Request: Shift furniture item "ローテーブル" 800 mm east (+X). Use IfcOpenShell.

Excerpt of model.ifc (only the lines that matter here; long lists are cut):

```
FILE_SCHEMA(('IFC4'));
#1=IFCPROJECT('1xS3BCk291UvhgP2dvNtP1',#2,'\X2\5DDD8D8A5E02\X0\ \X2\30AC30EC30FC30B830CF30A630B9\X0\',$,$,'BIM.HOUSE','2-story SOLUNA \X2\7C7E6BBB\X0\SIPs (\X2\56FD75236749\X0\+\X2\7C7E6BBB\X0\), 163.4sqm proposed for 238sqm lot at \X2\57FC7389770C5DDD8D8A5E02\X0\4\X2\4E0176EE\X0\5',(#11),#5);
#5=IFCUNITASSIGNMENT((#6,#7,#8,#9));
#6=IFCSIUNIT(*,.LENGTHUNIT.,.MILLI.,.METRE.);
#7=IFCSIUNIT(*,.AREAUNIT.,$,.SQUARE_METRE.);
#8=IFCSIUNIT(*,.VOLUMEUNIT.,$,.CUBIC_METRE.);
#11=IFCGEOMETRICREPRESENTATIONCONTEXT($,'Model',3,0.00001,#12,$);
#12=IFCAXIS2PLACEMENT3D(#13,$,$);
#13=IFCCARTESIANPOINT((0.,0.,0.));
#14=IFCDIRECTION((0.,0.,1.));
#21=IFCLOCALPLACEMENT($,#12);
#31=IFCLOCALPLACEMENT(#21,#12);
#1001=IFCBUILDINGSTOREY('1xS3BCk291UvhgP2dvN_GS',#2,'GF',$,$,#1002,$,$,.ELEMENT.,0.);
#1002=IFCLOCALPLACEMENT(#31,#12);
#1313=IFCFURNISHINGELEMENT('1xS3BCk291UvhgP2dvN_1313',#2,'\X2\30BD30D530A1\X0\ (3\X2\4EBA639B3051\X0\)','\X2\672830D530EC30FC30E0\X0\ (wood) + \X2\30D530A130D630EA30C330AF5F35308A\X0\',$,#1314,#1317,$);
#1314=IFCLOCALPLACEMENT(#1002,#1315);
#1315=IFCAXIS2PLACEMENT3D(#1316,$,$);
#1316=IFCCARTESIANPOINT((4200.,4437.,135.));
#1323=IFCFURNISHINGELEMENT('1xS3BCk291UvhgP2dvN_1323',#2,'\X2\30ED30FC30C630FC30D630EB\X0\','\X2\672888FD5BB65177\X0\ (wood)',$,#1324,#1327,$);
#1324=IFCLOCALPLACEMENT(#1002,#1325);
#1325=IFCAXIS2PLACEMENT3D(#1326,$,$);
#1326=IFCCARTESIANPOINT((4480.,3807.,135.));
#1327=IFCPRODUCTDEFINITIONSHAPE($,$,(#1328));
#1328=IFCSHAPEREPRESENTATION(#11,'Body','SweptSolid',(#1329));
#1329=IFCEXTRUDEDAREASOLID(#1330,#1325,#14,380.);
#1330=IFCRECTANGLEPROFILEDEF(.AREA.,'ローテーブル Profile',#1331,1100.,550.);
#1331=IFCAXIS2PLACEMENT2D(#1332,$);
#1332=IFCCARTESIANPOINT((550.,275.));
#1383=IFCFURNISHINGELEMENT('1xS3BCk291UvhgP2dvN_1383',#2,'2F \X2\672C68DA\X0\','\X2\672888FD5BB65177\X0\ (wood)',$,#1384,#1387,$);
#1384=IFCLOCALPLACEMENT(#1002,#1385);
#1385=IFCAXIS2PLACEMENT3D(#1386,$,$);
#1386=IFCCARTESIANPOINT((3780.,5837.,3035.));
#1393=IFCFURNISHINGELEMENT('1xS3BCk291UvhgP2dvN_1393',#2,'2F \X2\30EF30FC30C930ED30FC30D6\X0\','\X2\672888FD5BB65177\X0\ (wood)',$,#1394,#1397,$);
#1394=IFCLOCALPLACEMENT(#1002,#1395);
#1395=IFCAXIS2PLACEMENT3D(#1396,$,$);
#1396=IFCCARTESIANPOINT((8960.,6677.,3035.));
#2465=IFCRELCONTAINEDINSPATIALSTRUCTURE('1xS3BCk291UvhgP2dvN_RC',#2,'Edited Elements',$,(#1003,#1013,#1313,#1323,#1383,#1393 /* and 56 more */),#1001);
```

```python
import ifcopenshell
import ifcopenshell.api.geometry
import ifcopenshell.util.placement
import ifcopenshell.util.unit

model = ifcopenshell.open("model.ifc")
unit_scale = ifcopenshell.util.unit.calculate_unit_scale(model)

item = model.by_guid("1xS3BCk291UvhgP2dvN_1323")
matrix = ifcopenshell.util.placement.get_local_placement(item.ObjectPlacement)
matrix[0, 3] += 0.8 / unit_scale
ifcopenshell.api.geometry.edit_object_placement(model, product=item, matrix=matrix, is_si=False)

print(ifcopenshell.util.placement.get_local_placement(item.ObjectPlacement).round(3) + 0.0)

model.write("model-out.ifc")
```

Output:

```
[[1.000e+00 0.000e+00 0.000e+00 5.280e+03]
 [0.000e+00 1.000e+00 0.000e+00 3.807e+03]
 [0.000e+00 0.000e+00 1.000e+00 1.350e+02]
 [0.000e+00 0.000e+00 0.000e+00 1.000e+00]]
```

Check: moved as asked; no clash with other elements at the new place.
